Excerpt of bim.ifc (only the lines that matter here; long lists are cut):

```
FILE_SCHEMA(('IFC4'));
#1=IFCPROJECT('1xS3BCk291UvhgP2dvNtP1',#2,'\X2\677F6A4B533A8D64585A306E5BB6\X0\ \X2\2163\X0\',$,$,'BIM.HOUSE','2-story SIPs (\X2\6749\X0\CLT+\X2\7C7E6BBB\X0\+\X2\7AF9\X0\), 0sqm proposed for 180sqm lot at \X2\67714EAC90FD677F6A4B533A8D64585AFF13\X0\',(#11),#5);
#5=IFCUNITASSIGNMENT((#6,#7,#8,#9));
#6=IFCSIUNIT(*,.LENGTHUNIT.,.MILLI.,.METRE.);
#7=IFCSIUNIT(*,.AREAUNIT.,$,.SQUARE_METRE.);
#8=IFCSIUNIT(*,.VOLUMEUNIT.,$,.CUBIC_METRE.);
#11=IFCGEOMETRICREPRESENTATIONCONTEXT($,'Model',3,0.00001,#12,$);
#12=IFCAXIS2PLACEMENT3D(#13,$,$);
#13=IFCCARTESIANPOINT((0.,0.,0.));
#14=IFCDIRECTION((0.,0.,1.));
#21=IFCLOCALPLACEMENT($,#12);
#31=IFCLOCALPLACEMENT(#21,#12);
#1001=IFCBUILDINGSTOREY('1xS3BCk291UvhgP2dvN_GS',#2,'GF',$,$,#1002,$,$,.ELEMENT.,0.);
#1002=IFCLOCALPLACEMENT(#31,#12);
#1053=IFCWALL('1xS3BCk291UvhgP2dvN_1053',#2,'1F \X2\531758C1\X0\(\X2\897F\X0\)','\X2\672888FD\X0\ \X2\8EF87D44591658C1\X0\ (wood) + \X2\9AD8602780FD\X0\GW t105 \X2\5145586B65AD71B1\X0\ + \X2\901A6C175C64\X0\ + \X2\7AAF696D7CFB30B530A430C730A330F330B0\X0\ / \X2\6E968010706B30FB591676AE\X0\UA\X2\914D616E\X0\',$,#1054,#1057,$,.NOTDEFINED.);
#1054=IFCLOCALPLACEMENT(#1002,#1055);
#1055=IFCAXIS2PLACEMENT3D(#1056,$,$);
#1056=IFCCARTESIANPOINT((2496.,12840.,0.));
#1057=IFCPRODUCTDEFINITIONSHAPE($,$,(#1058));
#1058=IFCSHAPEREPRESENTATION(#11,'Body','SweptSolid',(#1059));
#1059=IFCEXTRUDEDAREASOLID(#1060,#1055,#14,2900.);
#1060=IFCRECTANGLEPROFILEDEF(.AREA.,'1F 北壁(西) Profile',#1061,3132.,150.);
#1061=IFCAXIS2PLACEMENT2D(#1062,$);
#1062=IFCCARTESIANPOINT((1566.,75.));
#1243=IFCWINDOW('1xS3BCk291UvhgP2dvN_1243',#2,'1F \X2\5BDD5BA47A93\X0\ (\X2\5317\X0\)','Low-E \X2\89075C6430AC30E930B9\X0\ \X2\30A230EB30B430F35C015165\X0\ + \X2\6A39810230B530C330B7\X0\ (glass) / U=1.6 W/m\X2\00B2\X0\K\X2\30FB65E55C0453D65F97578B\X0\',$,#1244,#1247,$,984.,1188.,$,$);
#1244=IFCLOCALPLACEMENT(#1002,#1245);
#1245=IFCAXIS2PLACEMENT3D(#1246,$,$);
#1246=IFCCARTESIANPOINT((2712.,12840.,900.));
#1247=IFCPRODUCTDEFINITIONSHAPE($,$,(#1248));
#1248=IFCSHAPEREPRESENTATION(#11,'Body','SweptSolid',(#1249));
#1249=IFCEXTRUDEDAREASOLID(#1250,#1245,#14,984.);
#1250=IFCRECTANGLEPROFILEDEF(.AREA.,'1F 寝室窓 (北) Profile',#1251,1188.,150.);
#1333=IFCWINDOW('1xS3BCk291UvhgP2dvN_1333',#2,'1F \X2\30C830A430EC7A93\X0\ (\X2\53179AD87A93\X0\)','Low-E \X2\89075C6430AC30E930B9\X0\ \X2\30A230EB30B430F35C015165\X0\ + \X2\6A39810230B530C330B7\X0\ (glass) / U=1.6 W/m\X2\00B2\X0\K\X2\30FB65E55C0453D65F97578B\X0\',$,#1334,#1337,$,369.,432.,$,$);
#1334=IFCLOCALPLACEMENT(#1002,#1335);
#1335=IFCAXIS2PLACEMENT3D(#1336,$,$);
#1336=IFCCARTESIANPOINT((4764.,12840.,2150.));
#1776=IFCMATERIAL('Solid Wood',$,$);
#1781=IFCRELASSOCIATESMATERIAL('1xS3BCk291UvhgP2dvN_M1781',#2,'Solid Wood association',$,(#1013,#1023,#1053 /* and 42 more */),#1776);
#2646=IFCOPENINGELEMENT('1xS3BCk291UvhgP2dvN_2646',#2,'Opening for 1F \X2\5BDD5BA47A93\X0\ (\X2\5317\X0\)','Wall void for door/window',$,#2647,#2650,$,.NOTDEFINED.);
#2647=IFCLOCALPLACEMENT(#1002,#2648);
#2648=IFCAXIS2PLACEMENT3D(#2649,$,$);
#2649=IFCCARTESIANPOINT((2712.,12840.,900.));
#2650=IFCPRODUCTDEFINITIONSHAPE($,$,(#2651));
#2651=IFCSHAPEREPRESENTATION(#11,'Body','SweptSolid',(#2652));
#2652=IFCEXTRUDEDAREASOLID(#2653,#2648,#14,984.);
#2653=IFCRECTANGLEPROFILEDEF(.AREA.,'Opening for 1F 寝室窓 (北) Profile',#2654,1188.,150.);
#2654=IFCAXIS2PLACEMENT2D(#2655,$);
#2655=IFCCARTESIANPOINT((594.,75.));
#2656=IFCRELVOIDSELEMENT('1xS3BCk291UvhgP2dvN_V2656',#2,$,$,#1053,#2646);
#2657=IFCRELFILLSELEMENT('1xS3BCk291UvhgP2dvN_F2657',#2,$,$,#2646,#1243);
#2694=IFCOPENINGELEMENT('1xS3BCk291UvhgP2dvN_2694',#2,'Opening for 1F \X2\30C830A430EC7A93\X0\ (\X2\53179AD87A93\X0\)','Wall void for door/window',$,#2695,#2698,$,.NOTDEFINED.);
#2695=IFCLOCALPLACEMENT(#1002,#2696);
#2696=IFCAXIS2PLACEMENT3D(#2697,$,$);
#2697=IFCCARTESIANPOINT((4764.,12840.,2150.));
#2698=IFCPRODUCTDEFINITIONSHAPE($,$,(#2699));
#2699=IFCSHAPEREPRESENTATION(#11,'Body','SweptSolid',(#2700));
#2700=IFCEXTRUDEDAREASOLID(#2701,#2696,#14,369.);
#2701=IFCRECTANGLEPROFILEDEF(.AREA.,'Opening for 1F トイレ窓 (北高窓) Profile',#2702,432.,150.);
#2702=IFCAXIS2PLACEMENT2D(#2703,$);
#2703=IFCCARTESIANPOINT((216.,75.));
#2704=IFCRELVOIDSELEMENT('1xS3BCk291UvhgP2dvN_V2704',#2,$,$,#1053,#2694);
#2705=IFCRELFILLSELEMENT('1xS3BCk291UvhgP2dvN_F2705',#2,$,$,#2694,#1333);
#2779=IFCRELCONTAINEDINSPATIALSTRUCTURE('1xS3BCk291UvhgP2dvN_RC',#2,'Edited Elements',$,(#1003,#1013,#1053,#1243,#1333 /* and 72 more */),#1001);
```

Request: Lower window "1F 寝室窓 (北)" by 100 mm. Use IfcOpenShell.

```python
import numpy as np
import ifcopenshell
import ifcopenshell.api.geometry
import ifcopenshell.util.placement
import ifcopenshell.util.unit

model = ifcopenshell.open("bim.ifc")
unit_scale = ifcopenshell.util.unit.calculate_unit_scale(model)

window = model.by_guid("1xS3BCk291UvhgP2dvN_1243")
opening = window.FillsVoids[0].RelatingOpeningElement
dz = -0.1 / unit_scale

shift = np.array([0.0, 0.0, dz])
# The window is not placed relative to its opening, so move both.
for product in (opening, window):
    matrix = ifcopenshell.util.placement.get_local_placement(product.ObjectPlacement)
    matrix[:3, 3] += shift
    ifcopenshell.api.geometry.edit_object_placement(model, product=product, matrix=matrix, is_si=False)

print(f"moved by {dz * unit_scale:+.3f} m")

model.write("bim_rev.ifc")
```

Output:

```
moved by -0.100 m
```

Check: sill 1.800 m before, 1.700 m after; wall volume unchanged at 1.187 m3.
